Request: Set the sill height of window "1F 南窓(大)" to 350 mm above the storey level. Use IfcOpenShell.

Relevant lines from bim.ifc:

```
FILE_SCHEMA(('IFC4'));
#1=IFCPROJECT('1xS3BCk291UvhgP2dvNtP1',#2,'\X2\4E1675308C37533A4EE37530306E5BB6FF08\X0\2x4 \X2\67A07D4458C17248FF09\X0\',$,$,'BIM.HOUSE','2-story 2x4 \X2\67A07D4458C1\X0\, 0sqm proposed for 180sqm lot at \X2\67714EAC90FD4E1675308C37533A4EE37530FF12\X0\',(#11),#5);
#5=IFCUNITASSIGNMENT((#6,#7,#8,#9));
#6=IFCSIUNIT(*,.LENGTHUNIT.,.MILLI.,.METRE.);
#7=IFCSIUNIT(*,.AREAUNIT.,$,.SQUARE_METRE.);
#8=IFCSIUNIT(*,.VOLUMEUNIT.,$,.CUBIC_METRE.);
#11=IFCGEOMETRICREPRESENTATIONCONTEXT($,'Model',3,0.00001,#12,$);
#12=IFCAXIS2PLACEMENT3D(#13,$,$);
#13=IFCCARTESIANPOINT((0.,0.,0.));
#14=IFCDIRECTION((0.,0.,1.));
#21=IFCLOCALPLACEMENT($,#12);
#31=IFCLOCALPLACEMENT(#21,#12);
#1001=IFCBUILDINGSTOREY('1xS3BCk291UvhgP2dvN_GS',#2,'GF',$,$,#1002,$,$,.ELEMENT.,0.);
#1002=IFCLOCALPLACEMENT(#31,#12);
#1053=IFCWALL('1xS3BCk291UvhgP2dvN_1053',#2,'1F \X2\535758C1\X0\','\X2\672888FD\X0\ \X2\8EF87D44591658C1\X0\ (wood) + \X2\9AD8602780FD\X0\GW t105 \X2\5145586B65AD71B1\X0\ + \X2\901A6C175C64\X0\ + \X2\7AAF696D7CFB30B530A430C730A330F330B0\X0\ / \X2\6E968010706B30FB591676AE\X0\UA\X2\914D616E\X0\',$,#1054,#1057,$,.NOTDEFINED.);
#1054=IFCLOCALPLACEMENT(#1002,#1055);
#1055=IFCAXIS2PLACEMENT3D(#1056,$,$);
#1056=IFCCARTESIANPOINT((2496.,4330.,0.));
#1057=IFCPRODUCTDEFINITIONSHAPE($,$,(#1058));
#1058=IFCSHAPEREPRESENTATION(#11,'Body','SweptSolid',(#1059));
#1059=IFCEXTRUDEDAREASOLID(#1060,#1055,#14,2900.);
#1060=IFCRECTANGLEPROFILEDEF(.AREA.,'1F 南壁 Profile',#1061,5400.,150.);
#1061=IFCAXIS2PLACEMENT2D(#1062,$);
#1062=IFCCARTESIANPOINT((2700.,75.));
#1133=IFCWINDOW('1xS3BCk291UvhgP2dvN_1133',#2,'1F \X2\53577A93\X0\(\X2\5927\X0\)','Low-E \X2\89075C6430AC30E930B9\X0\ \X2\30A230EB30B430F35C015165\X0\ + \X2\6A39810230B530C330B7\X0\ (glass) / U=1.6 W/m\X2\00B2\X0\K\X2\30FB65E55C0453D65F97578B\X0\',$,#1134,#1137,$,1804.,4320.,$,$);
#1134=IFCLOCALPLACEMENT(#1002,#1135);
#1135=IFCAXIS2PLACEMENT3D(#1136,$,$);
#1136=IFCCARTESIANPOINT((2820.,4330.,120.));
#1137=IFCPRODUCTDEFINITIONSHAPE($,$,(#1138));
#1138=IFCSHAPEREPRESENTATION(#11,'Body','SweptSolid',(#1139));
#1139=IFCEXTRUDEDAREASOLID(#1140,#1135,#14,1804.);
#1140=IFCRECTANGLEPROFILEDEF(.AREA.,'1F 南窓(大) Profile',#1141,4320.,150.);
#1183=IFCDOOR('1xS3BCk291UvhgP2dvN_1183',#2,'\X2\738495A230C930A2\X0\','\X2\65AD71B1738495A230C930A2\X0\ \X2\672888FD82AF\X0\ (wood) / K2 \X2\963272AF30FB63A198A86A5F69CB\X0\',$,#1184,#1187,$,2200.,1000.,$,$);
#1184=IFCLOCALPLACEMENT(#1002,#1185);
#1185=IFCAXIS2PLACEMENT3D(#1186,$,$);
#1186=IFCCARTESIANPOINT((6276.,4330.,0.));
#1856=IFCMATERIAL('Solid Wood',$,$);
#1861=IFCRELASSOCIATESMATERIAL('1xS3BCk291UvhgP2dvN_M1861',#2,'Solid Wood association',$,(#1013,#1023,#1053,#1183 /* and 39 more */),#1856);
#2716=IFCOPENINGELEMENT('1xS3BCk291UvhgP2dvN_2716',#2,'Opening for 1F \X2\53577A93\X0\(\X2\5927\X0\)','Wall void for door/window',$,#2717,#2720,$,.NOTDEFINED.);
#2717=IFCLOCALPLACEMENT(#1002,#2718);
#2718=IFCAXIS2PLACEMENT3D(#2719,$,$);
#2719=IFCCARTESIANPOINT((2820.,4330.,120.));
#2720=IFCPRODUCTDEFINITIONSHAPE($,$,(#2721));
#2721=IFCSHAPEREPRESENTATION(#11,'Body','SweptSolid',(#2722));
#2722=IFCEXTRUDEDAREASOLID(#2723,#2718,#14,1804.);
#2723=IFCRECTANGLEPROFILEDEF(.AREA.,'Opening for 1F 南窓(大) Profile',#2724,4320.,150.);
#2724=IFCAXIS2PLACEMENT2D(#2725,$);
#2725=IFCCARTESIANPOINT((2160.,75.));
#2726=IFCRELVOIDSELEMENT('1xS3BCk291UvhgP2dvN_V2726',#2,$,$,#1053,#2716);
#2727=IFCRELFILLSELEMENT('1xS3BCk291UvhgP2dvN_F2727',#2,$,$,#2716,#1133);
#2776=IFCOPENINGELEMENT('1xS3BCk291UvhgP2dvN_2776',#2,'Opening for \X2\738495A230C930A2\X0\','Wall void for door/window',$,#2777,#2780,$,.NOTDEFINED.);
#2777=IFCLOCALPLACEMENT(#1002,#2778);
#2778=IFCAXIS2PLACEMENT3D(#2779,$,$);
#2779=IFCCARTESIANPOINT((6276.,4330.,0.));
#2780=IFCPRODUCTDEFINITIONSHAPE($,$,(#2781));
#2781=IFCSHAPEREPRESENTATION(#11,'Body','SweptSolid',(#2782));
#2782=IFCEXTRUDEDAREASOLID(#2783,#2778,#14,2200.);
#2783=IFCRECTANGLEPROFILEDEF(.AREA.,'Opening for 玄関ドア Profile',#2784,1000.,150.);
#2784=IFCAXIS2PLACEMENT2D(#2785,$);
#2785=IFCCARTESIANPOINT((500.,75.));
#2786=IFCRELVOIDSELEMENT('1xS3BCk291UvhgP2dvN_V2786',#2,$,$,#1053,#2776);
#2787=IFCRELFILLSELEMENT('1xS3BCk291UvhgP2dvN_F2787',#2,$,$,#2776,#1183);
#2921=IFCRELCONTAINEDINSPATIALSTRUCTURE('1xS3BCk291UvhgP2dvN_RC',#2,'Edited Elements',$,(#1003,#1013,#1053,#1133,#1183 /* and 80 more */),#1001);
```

```python
import numpy as np
import ifcopenshell
import ifcopenshell.api.geometry
import ifcopenshell.geom
import ifcopenshell.util.element
import ifcopenshell.util.placement
import ifcopenshell.util.shape
import ifcopenshell.util.unit

model = ifcopenshell.open("bim.ifc")
unit_scale = ifcopenshell.util.unit.calculate_unit_scale(model)

window = model.by_id(1133)
opening = window.FillsVoids[0].RelatingOpeningElement
storey = ifcopenshell.util.element.get_container(window, ifc_class="IfcBuildingStorey")
level = ifcopenshell.util.placement.get_local_placement(storey.ObjectPlacement)[2, 3]

# The opening's origin need not be at the sill, so measure its lowest point.
shape = ifcopenshell.geom.create_shape(ifcopenshell.geom.settings(), opening)
bottom = ifcopenshell.util.shape.get_shape_bottom_elevation(shape, shape.geometry) / unit_scale
dz = level + 350.0 - bottom

shift = np.array([0.0, 0.0, dz])
# The window is not placed relative to its opening, so move both.
for product in (opening, window):
    matrix = ifcopenshell.util.placement.get_local_placement(product.ObjectPlacement)
    matrix[:3, 3] += shift
    ifcopenshell.api.geometry.edit_object_placement(model, product=product, matrix=matrix, is_si=False)

print(f"moved by {dz * unit_scale:+.3f} m")

model.write("bim-out.ifc")
```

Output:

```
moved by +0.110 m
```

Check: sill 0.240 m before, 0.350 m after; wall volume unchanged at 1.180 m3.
